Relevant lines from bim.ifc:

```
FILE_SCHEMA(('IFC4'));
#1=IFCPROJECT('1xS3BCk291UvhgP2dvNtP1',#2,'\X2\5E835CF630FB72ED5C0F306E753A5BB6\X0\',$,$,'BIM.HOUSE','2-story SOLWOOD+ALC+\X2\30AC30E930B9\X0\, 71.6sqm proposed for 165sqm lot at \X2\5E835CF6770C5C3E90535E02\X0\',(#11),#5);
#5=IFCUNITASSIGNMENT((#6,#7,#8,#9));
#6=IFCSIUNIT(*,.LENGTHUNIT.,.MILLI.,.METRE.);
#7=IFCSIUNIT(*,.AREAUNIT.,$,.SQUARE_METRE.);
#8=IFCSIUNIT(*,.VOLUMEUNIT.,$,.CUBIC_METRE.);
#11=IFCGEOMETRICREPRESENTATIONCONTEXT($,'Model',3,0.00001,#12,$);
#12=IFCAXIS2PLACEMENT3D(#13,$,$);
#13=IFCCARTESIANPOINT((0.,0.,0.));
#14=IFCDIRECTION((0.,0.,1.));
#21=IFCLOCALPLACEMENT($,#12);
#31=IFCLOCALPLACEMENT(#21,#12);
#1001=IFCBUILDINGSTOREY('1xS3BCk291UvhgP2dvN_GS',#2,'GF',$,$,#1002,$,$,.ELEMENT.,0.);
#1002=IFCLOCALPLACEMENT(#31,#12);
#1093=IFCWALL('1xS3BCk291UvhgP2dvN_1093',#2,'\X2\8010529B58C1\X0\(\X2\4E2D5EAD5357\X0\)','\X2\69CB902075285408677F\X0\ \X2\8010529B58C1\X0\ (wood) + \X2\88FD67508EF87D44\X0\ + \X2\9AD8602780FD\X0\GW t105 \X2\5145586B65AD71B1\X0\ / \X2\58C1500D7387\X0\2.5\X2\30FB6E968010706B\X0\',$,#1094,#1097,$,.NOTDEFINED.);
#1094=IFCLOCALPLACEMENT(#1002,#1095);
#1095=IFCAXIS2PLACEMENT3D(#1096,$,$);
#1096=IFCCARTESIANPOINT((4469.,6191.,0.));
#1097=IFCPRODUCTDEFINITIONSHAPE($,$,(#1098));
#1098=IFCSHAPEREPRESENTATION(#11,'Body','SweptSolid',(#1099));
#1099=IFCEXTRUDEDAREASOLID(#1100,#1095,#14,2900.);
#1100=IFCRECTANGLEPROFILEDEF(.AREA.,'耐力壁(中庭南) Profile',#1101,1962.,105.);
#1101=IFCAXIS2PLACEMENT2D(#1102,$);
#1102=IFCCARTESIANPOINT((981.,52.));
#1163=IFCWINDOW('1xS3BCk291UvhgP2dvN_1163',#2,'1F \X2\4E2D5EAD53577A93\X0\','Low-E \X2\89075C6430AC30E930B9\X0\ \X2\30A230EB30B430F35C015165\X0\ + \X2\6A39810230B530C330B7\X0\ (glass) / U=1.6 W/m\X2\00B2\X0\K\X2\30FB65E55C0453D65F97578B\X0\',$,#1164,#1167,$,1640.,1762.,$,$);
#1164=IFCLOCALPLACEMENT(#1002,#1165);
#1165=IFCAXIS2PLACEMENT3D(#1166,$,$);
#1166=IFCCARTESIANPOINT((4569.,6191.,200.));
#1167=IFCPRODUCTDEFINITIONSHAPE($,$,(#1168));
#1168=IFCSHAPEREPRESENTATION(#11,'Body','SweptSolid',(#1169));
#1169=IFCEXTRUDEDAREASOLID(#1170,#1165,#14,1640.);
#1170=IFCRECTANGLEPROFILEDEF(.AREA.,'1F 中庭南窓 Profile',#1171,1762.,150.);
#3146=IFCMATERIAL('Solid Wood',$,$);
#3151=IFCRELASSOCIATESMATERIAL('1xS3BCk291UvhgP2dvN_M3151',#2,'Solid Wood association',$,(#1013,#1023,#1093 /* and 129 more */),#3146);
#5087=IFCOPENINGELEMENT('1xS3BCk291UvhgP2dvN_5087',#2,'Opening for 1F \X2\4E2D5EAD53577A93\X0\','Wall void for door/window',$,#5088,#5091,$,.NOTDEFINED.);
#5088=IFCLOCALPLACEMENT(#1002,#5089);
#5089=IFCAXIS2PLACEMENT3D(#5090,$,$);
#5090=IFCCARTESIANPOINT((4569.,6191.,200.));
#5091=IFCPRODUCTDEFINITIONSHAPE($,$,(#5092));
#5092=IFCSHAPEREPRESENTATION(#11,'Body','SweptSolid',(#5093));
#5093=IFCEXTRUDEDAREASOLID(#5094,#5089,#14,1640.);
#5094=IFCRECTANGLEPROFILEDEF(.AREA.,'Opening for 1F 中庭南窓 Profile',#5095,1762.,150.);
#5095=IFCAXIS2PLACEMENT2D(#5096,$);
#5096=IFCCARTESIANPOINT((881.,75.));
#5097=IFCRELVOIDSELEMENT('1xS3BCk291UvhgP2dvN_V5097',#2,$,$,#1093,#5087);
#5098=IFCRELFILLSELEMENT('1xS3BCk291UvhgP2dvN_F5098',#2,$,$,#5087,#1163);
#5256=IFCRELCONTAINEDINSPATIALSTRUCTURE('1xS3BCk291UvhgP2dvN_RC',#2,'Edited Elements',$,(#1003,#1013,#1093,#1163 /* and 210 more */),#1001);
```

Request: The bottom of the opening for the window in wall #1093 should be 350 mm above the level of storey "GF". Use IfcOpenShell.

```python
import numpy as np
import ifcopenshell
import ifcopenshell.api.geometry
import ifcopenshell.geom
import ifcopenshell.util.element
import ifcopenshell.util.placement
import ifcopenshell.util.shape
import ifcopenshell.util.unit

model = ifcopenshell.open("bim.ifc")
unit_scale = ifcopenshell.util.unit.calculate_unit_scale(model)

window = model.by_id(1163)
opening = window.FillsVoids[0].RelatingOpeningElement
storey = ifcopenshell.util.element.get_container(window, ifc_class="IfcBuildingStorey")
level = ifcopenshell.util.placement.get_local_placement(storey.ObjectPlacement)[2, 3]

# The opening's origin need not be at the sill, so measure its lowest point.
shape = ifcopenshell.geom.create_shape(ifcopenshell.geom.settings(), opening)
bottom = ifcopenshell.util.shape.get_shape_bottom_elevation(shape, shape.geometry) / unit_scale
dz = level + 0.35 / unit_scale - bottom

shift = np.array([0.0, 0.0, dz])
# The window is not placed relative to its opening, so move both.
for product in (opening, window):
    matrix = ifcopenshell.util.placement.get_local_placement(product.ObjectPlacement)
    matrix[:3, 3] += shift
    ifcopenshell.api.geometry.edit_object_placement(model, product=product, matrix=matrix, is_si=False)

print(f"moved by {dz * unit_scale:+.3f} m")

model.write("bim_rev.ifc")
```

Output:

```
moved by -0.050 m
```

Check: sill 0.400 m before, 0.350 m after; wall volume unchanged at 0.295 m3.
